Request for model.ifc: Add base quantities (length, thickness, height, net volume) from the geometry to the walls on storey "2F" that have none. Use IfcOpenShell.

First a look at what the model holds.

```python
import ifcopenshell
import ifcopenshell.util.element
import ifcopenshell.util.unit

model = ifcopenshell.open("model.ifc")
print(model.schema)
for unit_type in ("LENGTHUNIT", "AREAUNIT", "VOLUMEUNIT"):
    print(unit_type, ifcopenshell.util.unit.calculate_unit_scale(model, unit_type))
storey = next(s for s in model.by_type("IfcBuildingStorey") if s.Name == "2F")
walls = [e for e in ifcopenshell.util.element.get_decomposition(storey) if e.is_a("IfcWall")]
for e in sorted(walls, key=lambda e: e.id()):
    print(e.id(), e.is_a(), e.Name, list(ifcopenshell.util.element.get_psets(e, qtos_only=True)), sep=" | ")
```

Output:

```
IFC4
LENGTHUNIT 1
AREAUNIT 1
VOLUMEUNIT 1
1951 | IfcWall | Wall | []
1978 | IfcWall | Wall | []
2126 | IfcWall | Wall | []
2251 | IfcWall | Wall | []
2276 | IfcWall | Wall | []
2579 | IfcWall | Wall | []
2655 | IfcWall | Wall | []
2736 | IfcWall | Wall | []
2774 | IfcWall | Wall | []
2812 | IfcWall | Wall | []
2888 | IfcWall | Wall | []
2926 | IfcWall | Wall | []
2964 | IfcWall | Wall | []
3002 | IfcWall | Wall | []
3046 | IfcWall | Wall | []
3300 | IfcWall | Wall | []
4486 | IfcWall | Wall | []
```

```python
import ifcopenshell
import ifcopenshell.api.pset
import ifcopenshell.geom
import ifcopenshell.util.element
import ifcopenshell.util.shape
import ifcopenshell.util.unit

model = ifcopenshell.open("model.ifc")
unit_scale = ifcopenshell.util.unit.calculate_unit_scale(model)
volume_scale = ifcopenshell.util.unit.calculate_unit_scale(model, "VOLUMEUNIT")
settings = ifcopenshell.geom.settings()

storey = next(s for s in model.by_type("IfcBuildingStorey") if s.Name == "2F")
walls = [e for e in ifcopenshell.util.element.get_decomposition(storey) if e.is_a("IfcWall")]

for e in sorted(walls, key=lambda e: e.id()):
    if ifcopenshell.util.element.get_psets(e, qtos_only=True, should_inherit=False):
        continue
    # Geometry comes back in metres, in the element's own axes.
    shape = ifcopenshell.geom.create_shape(settings, e)
    values = {
        "Length": ifcopenshell.util.shape.get_x(shape.geometry) / unit_scale,
        "Width": ifcopenshell.util.shape.get_y(shape.geometry) / unit_scale,
        "Height": ifcopenshell.util.shape.get_z(shape.geometry) / unit_scale,
        "NetVolume": ifcopenshell.util.shape.get_volume(shape.geometry) / volume_scale,
    }
    qto = ifcopenshell.api.pset.add_qto(model, product=e, name="Qto_WallBaseQuantities")
    ifcopenshell.api.pset.edit_qto(model, qto=qto, properties=values)
    print(e.id(), {k: round(v, 3) for k, v in values.items()})

model.write("model_v2.ifc")
```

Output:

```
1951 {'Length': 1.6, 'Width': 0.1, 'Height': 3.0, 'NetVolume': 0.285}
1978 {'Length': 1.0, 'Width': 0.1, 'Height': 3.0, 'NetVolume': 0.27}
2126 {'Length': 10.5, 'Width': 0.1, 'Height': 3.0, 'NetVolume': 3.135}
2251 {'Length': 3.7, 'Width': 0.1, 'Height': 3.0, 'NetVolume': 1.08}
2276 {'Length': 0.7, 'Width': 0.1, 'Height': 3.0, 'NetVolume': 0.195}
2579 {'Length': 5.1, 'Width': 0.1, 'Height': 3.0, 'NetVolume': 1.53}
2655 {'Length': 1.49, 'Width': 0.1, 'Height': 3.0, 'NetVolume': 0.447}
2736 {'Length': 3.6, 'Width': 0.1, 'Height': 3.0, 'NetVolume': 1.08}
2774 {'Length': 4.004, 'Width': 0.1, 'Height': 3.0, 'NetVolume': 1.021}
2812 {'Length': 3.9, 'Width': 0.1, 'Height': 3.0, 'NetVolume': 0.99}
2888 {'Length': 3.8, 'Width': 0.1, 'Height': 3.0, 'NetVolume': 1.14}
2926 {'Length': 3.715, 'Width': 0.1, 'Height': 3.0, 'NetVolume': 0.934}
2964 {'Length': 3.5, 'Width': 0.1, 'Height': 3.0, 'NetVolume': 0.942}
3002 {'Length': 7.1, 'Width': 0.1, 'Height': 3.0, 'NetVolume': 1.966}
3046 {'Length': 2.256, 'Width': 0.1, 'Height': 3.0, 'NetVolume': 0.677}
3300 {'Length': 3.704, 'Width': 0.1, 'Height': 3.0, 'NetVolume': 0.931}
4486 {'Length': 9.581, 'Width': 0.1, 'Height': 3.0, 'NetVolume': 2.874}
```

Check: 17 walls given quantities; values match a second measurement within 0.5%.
